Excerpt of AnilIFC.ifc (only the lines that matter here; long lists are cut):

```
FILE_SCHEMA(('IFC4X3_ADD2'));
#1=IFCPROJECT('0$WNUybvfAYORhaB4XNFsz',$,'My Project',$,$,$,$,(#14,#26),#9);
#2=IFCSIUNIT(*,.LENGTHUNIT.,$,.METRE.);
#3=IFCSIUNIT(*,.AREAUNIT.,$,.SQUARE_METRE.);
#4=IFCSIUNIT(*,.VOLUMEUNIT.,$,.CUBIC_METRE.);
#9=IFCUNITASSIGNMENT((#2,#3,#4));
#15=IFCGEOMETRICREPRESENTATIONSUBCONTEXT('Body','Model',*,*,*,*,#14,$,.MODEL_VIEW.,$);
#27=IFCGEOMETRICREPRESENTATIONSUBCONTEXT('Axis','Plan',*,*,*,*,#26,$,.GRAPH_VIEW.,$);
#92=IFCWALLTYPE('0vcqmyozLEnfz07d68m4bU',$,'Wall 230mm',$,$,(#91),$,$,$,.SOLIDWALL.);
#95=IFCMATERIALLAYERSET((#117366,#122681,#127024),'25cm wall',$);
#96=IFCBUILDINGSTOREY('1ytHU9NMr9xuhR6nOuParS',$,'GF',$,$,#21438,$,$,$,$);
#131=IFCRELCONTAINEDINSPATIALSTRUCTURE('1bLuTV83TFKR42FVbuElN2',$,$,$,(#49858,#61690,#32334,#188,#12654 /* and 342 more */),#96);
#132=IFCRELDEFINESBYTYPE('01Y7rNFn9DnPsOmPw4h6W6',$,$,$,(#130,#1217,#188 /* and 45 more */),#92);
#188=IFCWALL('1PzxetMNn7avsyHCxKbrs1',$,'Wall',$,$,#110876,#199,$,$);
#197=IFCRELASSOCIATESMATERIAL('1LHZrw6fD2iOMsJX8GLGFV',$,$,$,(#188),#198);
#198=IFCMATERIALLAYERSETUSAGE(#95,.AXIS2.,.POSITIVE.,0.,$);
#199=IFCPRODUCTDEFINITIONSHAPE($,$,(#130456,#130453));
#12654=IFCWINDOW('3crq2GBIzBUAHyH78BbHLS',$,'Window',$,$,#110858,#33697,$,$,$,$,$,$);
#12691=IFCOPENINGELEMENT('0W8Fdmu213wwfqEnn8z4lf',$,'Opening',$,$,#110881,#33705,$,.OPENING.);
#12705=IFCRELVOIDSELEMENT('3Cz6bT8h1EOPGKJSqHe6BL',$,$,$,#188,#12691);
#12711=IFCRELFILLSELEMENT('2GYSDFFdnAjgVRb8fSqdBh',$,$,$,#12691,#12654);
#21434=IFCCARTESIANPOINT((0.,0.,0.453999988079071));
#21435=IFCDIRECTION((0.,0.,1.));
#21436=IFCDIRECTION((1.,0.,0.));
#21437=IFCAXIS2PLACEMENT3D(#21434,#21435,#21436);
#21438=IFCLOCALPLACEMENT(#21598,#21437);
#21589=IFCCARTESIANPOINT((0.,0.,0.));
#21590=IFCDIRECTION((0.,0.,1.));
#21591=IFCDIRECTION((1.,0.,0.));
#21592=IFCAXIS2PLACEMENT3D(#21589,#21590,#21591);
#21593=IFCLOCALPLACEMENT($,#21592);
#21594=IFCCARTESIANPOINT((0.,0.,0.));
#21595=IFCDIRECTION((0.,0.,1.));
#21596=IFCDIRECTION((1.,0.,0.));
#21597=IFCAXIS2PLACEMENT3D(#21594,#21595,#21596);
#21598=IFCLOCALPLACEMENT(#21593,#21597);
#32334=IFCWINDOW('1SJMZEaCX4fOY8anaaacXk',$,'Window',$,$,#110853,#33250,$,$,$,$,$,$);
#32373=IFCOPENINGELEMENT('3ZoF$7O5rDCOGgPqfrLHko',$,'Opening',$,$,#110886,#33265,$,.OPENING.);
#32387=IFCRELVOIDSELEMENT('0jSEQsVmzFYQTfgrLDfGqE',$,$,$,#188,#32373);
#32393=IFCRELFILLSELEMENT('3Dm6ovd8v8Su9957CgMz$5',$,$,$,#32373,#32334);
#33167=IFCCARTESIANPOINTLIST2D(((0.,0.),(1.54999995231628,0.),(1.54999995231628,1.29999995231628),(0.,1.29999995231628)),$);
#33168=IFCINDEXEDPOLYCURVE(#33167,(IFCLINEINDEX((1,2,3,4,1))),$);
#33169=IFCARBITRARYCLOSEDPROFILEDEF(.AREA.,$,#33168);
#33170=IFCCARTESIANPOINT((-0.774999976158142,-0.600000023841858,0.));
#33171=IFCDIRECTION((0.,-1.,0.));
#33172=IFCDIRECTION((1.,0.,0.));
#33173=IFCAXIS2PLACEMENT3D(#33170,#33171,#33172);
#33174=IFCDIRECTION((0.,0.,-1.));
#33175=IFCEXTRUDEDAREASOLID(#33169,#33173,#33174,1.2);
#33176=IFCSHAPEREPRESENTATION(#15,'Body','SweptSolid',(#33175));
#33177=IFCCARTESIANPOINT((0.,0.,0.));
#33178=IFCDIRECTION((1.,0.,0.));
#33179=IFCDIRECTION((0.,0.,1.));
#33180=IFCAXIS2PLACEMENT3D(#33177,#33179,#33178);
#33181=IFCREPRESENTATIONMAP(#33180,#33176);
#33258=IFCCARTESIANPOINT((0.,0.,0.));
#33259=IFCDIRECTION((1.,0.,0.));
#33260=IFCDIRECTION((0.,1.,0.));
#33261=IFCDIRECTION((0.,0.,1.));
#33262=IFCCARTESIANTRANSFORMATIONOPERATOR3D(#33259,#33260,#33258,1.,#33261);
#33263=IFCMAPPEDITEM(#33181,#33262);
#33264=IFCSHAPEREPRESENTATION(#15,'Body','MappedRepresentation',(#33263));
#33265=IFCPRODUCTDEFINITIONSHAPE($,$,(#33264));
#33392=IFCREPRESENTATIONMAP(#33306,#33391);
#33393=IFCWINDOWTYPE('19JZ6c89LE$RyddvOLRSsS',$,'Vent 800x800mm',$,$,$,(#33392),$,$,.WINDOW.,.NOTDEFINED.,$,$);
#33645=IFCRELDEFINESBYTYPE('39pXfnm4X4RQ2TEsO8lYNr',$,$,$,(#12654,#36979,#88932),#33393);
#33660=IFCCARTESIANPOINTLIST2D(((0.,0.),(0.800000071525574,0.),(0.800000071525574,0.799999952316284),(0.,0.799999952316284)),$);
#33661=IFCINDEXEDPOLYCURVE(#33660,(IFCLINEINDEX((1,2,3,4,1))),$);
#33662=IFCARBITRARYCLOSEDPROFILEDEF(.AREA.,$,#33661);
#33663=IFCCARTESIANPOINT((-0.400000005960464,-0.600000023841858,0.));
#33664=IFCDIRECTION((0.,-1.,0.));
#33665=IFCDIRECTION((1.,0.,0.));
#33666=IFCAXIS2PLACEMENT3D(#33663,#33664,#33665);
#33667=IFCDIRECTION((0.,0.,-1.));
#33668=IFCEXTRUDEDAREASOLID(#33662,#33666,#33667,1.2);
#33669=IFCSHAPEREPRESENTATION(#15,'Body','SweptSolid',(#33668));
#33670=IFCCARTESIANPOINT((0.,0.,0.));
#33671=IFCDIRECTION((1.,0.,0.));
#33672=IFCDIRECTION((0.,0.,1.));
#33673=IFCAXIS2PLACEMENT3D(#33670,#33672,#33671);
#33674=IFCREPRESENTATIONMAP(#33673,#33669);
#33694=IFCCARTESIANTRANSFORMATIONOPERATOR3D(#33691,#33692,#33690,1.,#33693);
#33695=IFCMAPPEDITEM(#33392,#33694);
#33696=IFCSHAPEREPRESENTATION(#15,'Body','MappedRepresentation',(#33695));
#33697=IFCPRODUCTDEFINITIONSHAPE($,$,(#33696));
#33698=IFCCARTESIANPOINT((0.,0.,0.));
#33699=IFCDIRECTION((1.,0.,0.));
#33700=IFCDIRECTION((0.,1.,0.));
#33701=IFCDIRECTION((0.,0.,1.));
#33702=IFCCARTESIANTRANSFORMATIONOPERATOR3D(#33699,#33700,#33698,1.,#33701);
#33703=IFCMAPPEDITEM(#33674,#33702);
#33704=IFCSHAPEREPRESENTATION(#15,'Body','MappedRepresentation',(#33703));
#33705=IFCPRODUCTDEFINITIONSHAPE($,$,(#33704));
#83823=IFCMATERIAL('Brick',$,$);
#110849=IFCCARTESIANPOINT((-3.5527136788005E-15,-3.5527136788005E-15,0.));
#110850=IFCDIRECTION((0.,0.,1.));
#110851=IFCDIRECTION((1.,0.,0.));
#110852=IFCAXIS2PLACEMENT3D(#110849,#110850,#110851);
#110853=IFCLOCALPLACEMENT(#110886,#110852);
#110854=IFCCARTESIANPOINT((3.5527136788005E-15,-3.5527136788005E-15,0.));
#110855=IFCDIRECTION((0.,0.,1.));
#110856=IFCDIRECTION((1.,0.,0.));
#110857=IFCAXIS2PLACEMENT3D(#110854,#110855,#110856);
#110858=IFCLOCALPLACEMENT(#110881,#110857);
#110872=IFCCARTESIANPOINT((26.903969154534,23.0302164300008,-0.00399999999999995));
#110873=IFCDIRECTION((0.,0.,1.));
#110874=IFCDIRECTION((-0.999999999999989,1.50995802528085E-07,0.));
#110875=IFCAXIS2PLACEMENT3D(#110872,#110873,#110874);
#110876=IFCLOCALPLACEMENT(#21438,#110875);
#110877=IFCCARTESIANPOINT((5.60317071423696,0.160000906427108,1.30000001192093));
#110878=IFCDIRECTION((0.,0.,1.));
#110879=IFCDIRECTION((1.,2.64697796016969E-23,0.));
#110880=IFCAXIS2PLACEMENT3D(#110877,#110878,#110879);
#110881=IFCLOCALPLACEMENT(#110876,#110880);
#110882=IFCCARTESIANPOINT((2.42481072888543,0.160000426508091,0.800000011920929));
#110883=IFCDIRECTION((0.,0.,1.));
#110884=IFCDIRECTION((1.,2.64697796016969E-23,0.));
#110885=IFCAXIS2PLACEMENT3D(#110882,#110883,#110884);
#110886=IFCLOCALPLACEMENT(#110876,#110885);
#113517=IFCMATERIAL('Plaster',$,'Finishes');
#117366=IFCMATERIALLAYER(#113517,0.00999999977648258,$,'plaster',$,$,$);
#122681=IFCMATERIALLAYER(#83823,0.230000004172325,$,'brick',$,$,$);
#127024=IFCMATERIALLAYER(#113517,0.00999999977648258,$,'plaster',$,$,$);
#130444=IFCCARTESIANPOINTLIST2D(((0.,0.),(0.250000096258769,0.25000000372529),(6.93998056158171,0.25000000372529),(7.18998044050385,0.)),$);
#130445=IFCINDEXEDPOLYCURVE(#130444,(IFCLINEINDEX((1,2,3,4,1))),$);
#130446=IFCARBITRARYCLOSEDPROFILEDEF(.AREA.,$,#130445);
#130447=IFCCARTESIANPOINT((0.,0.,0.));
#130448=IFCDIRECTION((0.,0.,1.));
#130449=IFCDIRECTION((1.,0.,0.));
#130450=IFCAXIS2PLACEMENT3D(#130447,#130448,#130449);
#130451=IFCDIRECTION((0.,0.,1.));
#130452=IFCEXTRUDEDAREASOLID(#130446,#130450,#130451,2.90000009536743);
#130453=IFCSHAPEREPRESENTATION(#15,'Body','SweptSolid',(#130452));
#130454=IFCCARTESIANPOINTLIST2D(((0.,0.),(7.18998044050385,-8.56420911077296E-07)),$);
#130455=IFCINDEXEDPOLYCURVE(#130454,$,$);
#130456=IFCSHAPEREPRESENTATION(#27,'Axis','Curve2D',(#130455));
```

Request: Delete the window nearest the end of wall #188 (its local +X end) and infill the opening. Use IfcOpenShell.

```python
import ifcopenshell
import ifcopenshell.api.feature
import ifcopenshell.api.root
import ifcopenshell.geom
import ifcopenshell.util.shape

model = ifcopenshell.open("AnilIFC.ifc")
settings = ifcopenshell.geom.settings()


def volume(element):
    """Net volume in cubic metres, openings subtracted."""
    shape = ifcopenshell.geom.create_shape(settings, element)
    return ifcopenshell.util.shape.get_volume(shape.geometry)


window = model.by_guid("3crq2GBIzBUAHyH78BbHLS")
opening = window.FillsVoids[0].RelatingOpeningElement
wall = opening.VoidsElements[0].RelatingBuildingElement
before = volume(wall)

ifcopenshell.api.root.remove_product(model, product=window)
ifcopenshell.api.feature.remove_feature(model, feature=opening)

after = volume(wall)

print(f"wall volume {before:.3f} -> {after:.3f} m3")

model.write("AnilIFC-out.ifc")
```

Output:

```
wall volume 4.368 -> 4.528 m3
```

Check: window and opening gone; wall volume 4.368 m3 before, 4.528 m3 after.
